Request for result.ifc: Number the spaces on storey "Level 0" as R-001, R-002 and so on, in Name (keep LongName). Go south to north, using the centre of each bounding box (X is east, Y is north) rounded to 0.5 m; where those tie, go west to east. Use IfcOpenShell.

First a look at what the model holds.

```python
import ifcopenshell
import ifcopenshell.util.element
import ifcopenshell.util.placement

model = ifcopenshell.open("result.ifc")
print(model.schema)
storey = next(s for s in model.by_type("IfcBuildingStorey") if s.Name == "Level 0")
spaces = [e for e in ifcopenshell.util.element.get_decomposition(storey) if e.is_a("IfcSpace")]
for e in sorted(spaces, key=lambda e: e.id()):
    origin = ifcopenshell.util.placement.get_local_placement(e.ObjectPlacement)[:3, 3]
    print(e.id(), e.Name, e.LongName, origin.round(2) + 0.0, sep=" | ")
```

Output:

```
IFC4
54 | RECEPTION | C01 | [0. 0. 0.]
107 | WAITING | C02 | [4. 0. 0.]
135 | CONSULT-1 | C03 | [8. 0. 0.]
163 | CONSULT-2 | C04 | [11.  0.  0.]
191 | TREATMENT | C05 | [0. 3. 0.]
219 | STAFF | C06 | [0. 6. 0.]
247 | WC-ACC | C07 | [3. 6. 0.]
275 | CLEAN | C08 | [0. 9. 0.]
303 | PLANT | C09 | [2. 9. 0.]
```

```python
import ifcopenshell
import ifcopenshell.geom
import ifcopenshell.util.element
import ifcopenshell.util.shape

model = ifcopenshell.open("result.ifc")
settings = ifcopenshell.geom.settings()
settings.set("use-world-coords", True)


def centre(element):
    shape = ifcopenshell.geom.create_shape(settings, element)
    return ifcopenshell.util.shape.get_bbox_centroid(shape.geometry)


storey = next(s for s in model.by_type("IfcBuildingStorey") if s.Name == "Level 0")
spaces = [e for e in ifcopenshell.util.element.get_decomposition(storey) if e.is_a("IfcSpace")]

# Insertion points can sit at a corner or the storey origin, so sort by the geometry (in metres).
centres = {e: centre(e) for e in spaces}
spaces.sort(key=lambda e: (round(centres[e][1] / 0.5), centres[e][0]))

for i, e in enumerate(spaces, start=1):
    number = f"R-0{i:02d}"
    e.Name = number
    print(e.id(), number)

model.write("result-out.ifc")
```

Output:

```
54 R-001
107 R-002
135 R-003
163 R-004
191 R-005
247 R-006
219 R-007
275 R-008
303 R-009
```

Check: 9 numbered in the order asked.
